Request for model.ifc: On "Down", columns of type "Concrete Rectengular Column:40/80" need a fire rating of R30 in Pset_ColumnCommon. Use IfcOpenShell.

First a look at what the model holds.

```python
import ifcopenshell
import ifcopenshell.util.element

model = ifcopenshell.open("model.ifc")
print(model.schema)
storey = next(s for s in model.by_type("IfcBuildingStorey") if s.Name == "Down")
columns = [e for e in ifcopenshell.util.element.get_decomposition(storey) if e.is_a("IfcColumn")]
seen = {}
for e in columns:
    element_type = ifcopenshell.util.element.get_type(e)
    key = (element_type.Name if element_type != e and element_type else None, ifcopenshell.util.element.get_pset(e, "Pset_ColumnCommon", "FireRating"))
    seen[key] = seen.get(key, 0) + 1
for (name, value), count in sorted(seen.items(), key=str):
    print(count, "x", name, "|", value)
```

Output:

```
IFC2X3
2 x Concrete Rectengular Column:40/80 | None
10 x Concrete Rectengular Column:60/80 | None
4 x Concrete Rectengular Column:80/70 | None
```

```python
import ifcopenshell
import ifcopenshell.api.pset
import ifcopenshell.util.element

model = ifcopenshell.open("model.ifc")

storey = next(s for s in model.by_type("IfcBuildingStorey") if s.Name == "Down")
columns = [e for e in ifcopenshell.util.element.get_decomposition(storey) if e.is_a("IfcColumn")]

count = 0
for e in columns:
    element_type = ifcopenshell.util.element.get_type(e)
    if element_type in (None, e) or element_type.Name != "Concrete Rectengular Column:40/80":
        continue
    # add_pset returns the element's existing set when there is one.
    pset = ifcopenshell.api.pset.add_pset(model, product=e, name="Pset_ColumnCommon")
    ifcopenshell.api.pset.edit_pset(model, pset=pset, properties={"FireRating": "R30"})
    count += 1

print(count, "columns updated")

model.write("model-out.ifc")
```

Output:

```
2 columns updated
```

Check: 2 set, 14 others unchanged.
